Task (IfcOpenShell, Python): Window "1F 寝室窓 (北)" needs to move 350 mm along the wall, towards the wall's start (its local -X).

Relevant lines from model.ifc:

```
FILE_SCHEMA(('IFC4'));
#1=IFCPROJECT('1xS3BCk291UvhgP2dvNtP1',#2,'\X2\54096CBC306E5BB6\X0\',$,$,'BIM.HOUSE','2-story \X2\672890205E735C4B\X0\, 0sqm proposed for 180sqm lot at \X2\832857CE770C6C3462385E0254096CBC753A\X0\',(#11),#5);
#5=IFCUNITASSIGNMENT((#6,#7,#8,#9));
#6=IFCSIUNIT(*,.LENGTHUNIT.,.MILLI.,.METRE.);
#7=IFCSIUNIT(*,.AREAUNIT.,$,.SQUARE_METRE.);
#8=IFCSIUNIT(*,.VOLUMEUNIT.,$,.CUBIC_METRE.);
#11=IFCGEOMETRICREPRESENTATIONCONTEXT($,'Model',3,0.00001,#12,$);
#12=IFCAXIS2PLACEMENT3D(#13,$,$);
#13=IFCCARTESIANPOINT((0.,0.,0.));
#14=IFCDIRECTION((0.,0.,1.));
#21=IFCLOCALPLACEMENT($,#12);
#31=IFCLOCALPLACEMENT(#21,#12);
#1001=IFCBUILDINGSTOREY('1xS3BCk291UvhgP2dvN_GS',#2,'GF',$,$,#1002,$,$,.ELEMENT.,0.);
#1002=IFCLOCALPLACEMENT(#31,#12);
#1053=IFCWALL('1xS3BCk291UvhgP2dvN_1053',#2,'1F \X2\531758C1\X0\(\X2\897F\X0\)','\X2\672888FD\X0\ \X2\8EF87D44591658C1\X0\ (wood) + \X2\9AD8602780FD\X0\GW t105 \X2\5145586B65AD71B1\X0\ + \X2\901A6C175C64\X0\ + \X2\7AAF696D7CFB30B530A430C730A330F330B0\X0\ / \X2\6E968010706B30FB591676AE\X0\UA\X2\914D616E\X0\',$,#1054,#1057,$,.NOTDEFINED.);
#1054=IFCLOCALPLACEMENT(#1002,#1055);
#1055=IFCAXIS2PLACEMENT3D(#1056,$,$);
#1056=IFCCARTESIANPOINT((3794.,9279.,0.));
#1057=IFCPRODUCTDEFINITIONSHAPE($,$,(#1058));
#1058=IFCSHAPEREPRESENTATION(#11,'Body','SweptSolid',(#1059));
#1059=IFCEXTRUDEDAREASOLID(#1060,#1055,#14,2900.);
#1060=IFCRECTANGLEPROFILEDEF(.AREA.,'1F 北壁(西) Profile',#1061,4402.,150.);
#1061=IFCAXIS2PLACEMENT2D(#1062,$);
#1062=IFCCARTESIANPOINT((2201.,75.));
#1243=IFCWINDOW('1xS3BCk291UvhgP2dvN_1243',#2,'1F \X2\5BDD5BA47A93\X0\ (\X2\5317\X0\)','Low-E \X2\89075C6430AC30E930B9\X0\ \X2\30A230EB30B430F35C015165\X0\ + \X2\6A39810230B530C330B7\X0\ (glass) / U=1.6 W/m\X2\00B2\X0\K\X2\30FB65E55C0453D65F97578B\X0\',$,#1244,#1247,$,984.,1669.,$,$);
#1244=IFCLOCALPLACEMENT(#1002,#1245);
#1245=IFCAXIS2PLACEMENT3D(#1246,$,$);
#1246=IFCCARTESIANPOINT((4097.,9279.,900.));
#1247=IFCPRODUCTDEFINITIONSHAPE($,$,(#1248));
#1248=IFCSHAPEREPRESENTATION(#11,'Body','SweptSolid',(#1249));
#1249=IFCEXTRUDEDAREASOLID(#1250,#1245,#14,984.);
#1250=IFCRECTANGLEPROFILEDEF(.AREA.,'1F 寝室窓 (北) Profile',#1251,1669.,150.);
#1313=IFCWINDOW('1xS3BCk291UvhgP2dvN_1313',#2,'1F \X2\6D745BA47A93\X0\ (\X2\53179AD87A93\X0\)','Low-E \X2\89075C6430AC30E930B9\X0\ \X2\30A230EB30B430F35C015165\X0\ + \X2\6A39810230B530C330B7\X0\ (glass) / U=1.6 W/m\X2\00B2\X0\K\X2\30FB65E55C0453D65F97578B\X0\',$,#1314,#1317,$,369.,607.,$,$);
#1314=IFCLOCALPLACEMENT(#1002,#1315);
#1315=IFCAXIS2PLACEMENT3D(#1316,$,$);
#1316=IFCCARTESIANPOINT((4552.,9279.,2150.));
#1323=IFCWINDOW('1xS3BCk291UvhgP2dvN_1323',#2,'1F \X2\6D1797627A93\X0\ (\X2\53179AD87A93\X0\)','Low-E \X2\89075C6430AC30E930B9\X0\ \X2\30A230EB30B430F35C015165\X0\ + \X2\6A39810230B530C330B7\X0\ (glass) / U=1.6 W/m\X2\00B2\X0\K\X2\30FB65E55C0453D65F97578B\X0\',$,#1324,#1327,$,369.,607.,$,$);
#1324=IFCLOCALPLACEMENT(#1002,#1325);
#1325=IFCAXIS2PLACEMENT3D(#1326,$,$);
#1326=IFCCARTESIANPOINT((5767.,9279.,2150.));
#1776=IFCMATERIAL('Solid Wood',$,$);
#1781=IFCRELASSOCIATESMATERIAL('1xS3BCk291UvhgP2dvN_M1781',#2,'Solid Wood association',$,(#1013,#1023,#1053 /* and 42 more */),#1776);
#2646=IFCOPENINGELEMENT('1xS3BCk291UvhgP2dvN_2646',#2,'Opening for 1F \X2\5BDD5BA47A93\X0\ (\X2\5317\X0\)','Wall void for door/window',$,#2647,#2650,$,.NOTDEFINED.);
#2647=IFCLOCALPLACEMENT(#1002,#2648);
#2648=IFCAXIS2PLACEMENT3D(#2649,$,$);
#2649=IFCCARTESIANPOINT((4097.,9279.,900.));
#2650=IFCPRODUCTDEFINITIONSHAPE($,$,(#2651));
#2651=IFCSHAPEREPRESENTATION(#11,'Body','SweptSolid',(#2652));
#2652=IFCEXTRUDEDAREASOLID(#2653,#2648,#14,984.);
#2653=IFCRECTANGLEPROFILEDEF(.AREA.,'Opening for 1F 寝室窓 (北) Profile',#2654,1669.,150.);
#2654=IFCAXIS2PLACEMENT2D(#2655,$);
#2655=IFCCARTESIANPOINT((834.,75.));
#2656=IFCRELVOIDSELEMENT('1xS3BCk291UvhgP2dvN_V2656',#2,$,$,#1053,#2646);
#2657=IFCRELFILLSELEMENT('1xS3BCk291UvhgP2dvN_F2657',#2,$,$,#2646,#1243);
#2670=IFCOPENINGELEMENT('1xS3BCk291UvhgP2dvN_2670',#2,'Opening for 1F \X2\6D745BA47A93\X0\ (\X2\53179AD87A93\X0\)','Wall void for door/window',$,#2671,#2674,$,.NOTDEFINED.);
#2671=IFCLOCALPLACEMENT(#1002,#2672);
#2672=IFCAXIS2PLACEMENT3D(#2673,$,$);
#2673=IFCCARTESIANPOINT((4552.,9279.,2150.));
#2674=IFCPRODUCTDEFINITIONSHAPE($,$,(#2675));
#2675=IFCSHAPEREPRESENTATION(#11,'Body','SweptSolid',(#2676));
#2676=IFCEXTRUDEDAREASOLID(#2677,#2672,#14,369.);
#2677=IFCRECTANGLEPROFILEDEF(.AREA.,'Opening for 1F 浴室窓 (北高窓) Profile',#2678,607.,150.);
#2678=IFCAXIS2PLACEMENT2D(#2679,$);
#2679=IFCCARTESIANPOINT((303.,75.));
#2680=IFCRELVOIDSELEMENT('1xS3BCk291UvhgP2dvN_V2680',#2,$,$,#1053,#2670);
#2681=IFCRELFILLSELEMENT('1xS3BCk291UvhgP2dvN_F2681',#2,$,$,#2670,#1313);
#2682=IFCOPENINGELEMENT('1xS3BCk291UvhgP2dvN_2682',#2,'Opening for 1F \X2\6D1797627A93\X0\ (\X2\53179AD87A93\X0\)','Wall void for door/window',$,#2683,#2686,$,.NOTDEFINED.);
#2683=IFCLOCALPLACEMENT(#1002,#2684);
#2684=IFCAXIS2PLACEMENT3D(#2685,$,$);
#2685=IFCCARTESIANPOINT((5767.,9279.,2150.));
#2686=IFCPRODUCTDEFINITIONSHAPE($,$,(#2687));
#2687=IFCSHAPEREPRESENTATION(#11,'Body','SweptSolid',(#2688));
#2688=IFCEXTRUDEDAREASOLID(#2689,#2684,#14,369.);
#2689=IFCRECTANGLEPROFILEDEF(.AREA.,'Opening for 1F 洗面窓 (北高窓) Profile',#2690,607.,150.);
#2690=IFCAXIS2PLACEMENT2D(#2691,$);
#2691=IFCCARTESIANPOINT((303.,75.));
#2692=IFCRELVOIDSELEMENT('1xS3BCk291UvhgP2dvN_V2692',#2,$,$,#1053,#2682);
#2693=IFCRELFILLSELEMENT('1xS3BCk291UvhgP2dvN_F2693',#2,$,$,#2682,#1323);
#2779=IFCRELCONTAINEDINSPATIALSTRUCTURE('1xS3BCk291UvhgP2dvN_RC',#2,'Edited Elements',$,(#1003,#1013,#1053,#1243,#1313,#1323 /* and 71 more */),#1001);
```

```python
import ifcopenshell
import ifcopenshell.api.geometry
import ifcopenshell.util.placement
import ifcopenshell.util.unit

model = ifcopenshell.open("model.ifc")
unit_scale = ifcopenshell.util.unit.calculate_unit_scale(model)

window = model.by_id(1243)
opening = window.FillsVoids[0].RelatingOpeningElement
wall = opening.VoidsElements[0].RelatingBuildingElement

wall_matrix = ifcopenshell.util.placement.get_local_placement(wall.ObjectPlacement)
shift = wall_matrix[:3, 0] * -0.35 / unit_scale
before = ifcopenshell.util.placement.get_local_placement(window.ObjectPlacement)[:3, 3].copy()

# The window is not placed relative to its opening, so move both.
for product in (opening, window):
    matrix = ifcopenshell.util.placement.get_local_placement(product.ObjectPlacement)
    matrix[:3, 3] += shift
    ifcopenshell.api.geometry.edit_object_placement(model, product=product, matrix=matrix, is_si=False)

after = ifcopenshell.util.placement.get_local_placement(window.ObjectPlacement)[:3, 3]
print("window moved by", (after - before).round(3) + 0.0)

model.write("model_rev.ifc")
```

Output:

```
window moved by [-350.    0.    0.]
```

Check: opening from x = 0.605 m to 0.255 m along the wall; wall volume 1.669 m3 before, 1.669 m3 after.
